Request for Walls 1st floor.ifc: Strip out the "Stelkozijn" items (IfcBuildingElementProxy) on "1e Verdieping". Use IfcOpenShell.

First a look at what the model holds.

```python
import ifcopenshell
import ifcopenshell.util.element

model = ifcopenshell.open("Walls 1st floor.ifc")
print(model.schema)
storey = next(s for s in model.by_type("IfcBuildingStorey") if s.Name == "1e Verdieping")
proxies = [e for e in ifcopenshell.util.element.get_decomposition(storey) if e.is_a("IfcBuildingElementProxy")]
seen = {}
for e in proxies:
    element_type = ifcopenshell.util.element.get_type(e)
    name = element_type.Name if element_type not in (None, e) else None
    seen[name] = seen.get(name, 0) + 1
for name, count in sorted(seen.items(), key=str):
    print(count, "x", name)
```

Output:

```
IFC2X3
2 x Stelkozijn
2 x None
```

```python
import ifcopenshell
import ifcopenshell.api.root
import ifcopenshell.util.element

model = ifcopenshell.open("Walls 1st floor.ifc")

storey = next(s for s in model.by_type("IfcBuildingStorey") if s.Name == "1e Verdieping")
proxies = [e for e in ifcopenshell.util.element.get_decomposition(storey) if e.is_a("IfcBuildingElementProxy")]
targets = [e for e in proxies if (t := ifcopenshell.util.element.get_type(e)) not in (None, e) and t.Name == "Stelkozijn"]

for e in targets:
    ifcopenshell.api.root.remove_product(model, product=e)
print(len(targets), "removed")

model.write("Walls 1st floor_edited.ifc")
```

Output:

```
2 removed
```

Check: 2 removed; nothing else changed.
